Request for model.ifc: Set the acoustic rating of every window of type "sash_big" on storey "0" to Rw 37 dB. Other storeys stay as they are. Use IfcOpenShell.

First a look at what the model holds.

```python
import ifcopenshell
import ifcopenshell.util.element

model = ifcopenshell.open("model.ifc")
print(model.schema)
storey = next(s for s in model.by_type("IfcBuildingStorey") if s.Name == "0")
windows = [e for e in ifcopenshell.util.element.get_decomposition(storey) if e.is_a("IfcWindow")]
seen = {}
for e in windows:
    element_type = ifcopenshell.util.element.get_type(e)
    key = (element_type.Name if element_type != e and element_type else None, ifcopenshell.util.element.get_pset(e, "Pset_WindowCommon", "AcousticRating"))
    seen[key] = seen.get(key, 0) + 1
for (name, value), count in sorted(seen.items(), key=str):
    print(count, "x", name, "|", value)
```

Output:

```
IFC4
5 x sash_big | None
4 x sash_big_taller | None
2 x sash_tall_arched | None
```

```python
import ifcopenshell
import ifcopenshell.api.pset
import ifcopenshell.util.element

model = ifcopenshell.open("model.ifc")

storey = next(s for s in model.by_type("IfcBuildingStorey") if s.Name == "0")
windows = [e for e in ifcopenshell.util.element.get_decomposition(storey) if e.is_a("IfcWindow")]

count = 0
for e in windows:
    element_type = ifcopenshell.util.element.get_type(e)
    if element_type in (None, e) or element_type.Name != "sash_big":
        continue
    # add_pset returns the element's existing set when there is one.
    pset = ifcopenshell.api.pset.add_pset(model, product=e, name="Pset_WindowCommon")
    ifcopenshell.api.pset.edit_pset(model, pset=pset, properties={"AcousticRating": "Rw 37 dB"})
    count += 1

print(count, "windows updated")

model.write("model_rev.ifc")
```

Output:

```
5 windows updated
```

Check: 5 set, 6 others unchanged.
